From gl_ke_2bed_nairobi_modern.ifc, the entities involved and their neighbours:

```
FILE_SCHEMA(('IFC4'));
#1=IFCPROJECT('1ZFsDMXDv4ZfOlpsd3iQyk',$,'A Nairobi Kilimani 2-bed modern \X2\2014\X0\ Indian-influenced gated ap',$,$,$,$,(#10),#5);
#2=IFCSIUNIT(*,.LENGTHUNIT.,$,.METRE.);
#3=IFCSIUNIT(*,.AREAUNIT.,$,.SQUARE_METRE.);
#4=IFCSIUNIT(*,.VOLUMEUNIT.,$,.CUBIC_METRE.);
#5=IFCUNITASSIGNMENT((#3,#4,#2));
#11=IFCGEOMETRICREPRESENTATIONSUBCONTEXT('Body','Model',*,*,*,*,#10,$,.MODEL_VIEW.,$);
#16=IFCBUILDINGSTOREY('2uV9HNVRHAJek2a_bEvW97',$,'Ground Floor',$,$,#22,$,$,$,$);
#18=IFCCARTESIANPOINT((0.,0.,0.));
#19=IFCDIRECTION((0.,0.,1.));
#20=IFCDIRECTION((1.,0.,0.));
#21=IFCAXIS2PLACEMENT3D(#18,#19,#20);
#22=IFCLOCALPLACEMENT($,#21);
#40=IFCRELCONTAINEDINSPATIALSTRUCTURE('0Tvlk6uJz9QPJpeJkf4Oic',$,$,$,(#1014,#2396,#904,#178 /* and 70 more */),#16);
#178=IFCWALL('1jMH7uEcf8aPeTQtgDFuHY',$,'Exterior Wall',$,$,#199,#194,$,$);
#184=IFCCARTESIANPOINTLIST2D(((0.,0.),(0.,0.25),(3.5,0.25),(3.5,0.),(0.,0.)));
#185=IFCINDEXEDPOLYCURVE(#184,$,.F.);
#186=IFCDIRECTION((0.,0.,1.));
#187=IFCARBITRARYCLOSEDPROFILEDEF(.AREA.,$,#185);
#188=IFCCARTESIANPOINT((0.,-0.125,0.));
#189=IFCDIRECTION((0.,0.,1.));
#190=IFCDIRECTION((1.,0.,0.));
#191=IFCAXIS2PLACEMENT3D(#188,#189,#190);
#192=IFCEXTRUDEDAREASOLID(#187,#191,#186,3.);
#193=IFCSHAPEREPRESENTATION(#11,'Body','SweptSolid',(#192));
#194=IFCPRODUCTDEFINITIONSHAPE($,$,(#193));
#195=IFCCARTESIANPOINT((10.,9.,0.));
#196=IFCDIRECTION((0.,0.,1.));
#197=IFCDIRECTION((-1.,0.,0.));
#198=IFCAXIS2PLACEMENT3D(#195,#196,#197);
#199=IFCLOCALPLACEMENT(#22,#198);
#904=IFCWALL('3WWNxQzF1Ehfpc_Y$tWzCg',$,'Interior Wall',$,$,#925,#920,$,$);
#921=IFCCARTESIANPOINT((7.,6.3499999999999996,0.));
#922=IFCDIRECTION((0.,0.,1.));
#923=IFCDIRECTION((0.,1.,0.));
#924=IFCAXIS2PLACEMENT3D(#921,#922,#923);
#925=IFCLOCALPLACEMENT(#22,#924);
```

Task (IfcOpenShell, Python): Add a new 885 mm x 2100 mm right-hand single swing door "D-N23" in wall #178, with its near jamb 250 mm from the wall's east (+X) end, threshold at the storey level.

```python
import numpy as np
import ifcopenshell
import ifcopenshell.api.feature
import ifcopenshell.api.geometry
import ifcopenshell.api.root
import ifcopenshell.api.spatial
import ifcopenshell.geom
import ifcopenshell.util.element
import ifcopenshell.util.placement
import ifcopenshell.util.representation
import ifcopenshell.util.shape
import ifcopenshell.util.unit

model = ifcopenshell.open("gl_ke_2bed_nairobi_modern.ifc")
unit_scale = ifcopenshell.util.unit.calculate_unit_scale(model)
settings = ifcopenshell.geom.settings()


def volume(element):
    """Net volume in cubic metres, openings subtracted."""
    shape = ifcopenshell.geom.create_shape(settings, element)
    return ifcopenshell.util.shape.get_volume(shape.geometry)


wall = model.by_guid("1jMH7uEcf8aPeTQtgDFuHY")
storey = ifcopenshell.util.element.get_container(wall, ifc_class="IfcBuildingStorey")
context = ifcopenshell.util.representation.get_context(model, "Model", "Body", "MODEL_VIEW")
before = volume(wall)

width, height, from_end, sill = 0.885, 2.1, 0.25, 0.0  # metres

# The wall runs along its own X axis, and the end named is its -X end.
wall_shape = ifcopenshell.geom.create_shape(settings, wall)
x, y, z = ifcopenshell.util.shape.get_vertices(wall_shape.geometry).T
start = x.min() + from_end
face, thickness = float(y.min()), float(y.max() - y.min())
wall_matrix = ifcopenshell.util.placement.get_local_placement(wall.ObjectPlacement)
level = ifcopenshell.util.placement.get_local_placement(storey.ObjectPlacement)[2, 3]


def in_wall(x, y):
    """Placement at x, y metres in the wall's axes, at sill height."""
    matrix = wall_matrix.copy()
    matrix[:, 3] = wall_matrix @ np.array([x / unit_scale, y / unit_scale, 0.0, 1.0])
    matrix[2, 3] = level + sill / unit_scale
    return matrix


# Opening: a box that overshoots both wall faces by 50 mm.
opening = ifcopenshell.api.root.create_entity(model, ifc_class="IfcOpeningElement", predefined_type="OPENING")
box = ifcopenshell.api.geometry.add_wall_representation(
    model, context=context, length=width, height=height, thickness=thickness + 0.1
)
ifcopenshell.api.geometry.assign_representation(model, product=opening, representation=box)
ifcopenshell.api.geometry.edit_object_placement(model, product=opening, matrix=in_wall(start, face - 0.05), is_si=False)
ifcopenshell.api.feature.add_feature(model, feature=opening, element=wall)

door = ifcopenshell.api.root.create_entity(model, ifc_class="IfcDoor", name="D-N23", predefined_type="DOOR")
door.OverallWidth, door.OverallHeight = width / unit_scale, height / unit_scale
door.OperationType = "SINGLE_SWING_RIGHT"
body = ifcopenshell.api.geometry.add_door_representation(
    model,
    context=context,
    overall_width=door.OverallWidth,
    overall_height=door.OverallHeight,
    operation_type="SINGLE_SWING_RIGHT",
    lining_properties={"LiningDepth": thickness / unit_scale, "ThresholdDepth": thickness / unit_scale},
)
ifcopenshell.api.geometry.assign_representation(model, product=door, representation=body)
ifcopenshell.api.spatial.assign_container(model, products=[door], relating_structure=storey)
ifcopenshell.api.feature.add_filling(model, opening=opening, element=door)

# The lining spans the wall, so the door starts at the wall face.
ifcopenshell.api.geometry.edit_object_placement(model, product=door, matrix=in_wall(start, face), is_si=False)

after = volume(wall)

print(f"wall volume {before:.3f} -> {after:.3f} m3")

model.write("gl_ke_2bed_nairobi_modern_v2.ifc")
```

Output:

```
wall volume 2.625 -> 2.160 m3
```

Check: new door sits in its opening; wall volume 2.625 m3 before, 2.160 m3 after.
